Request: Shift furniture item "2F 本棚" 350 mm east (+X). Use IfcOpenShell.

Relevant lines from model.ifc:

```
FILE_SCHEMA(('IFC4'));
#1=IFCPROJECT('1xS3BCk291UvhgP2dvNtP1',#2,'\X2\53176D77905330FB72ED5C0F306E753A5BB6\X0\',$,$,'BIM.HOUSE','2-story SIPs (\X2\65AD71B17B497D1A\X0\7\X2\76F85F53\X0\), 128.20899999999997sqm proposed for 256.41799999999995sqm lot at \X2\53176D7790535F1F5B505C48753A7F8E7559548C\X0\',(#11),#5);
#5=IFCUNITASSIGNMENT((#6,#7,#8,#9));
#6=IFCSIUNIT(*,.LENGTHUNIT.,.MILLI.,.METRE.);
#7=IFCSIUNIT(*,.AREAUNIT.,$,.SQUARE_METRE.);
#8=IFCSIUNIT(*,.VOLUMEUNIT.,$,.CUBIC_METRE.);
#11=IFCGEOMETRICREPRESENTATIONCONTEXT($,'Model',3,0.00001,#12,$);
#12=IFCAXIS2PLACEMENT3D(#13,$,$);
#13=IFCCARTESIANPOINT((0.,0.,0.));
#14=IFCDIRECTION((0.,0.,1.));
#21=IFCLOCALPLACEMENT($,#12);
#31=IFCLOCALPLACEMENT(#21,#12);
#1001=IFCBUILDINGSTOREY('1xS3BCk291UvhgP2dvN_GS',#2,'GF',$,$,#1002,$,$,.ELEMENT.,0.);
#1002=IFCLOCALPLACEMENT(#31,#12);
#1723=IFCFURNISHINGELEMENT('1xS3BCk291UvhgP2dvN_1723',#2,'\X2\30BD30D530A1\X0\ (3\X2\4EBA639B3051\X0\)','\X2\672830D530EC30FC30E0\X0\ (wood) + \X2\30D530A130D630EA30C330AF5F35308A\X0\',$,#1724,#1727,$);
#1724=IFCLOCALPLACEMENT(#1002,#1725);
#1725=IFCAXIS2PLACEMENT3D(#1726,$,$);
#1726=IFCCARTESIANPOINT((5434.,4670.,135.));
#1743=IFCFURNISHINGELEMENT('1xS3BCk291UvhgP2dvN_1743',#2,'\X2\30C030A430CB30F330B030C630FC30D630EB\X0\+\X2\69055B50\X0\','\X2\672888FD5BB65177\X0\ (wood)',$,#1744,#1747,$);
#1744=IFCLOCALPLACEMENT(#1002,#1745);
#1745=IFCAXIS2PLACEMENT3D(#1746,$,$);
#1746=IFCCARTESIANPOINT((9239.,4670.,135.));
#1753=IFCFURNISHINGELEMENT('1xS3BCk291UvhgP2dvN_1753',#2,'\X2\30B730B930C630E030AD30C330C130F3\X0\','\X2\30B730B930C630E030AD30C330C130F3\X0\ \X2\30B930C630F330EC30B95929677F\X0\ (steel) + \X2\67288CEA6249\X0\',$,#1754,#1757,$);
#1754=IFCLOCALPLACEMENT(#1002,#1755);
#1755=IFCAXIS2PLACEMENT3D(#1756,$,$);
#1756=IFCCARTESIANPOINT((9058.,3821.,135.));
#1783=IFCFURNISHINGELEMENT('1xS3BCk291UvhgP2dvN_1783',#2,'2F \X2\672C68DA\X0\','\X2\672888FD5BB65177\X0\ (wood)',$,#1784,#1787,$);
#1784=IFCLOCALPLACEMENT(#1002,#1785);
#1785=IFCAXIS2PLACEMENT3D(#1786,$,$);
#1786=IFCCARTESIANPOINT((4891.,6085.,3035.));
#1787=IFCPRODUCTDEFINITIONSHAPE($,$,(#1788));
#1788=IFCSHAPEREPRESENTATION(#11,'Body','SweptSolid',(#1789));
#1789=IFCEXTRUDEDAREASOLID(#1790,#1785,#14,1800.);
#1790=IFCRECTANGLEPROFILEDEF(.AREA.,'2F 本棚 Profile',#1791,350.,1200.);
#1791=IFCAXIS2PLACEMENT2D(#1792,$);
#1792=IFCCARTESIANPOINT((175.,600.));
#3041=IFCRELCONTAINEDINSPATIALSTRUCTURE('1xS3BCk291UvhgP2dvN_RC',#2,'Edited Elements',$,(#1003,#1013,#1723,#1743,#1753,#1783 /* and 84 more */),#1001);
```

```python
import ifcopenshell
import ifcopenshell.api.geometry
import ifcopenshell.util.placement
import ifcopenshell.util.unit

model = ifcopenshell.open("model.ifc")
unit_scale = ifcopenshell.util.unit.calculate_unit_scale(model)

item = model.by_id(1783)
matrix = ifcopenshell.util.placement.get_local_placement(item.ObjectPlacement)
matrix[0, 3] += 0.35 / unit_scale
ifcopenshell.api.geometry.edit_object_placement(model, product=item, matrix=matrix, is_si=False)

print(ifcopenshell.util.placement.get_local_placement(item.ObjectPlacement).round(3) + 0.0)

model.write("model_rev.ifc")
```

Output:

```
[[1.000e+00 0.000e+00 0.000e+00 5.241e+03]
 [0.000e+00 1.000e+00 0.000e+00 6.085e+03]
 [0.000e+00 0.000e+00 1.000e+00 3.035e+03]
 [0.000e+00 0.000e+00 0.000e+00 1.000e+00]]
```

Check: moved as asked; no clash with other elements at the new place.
